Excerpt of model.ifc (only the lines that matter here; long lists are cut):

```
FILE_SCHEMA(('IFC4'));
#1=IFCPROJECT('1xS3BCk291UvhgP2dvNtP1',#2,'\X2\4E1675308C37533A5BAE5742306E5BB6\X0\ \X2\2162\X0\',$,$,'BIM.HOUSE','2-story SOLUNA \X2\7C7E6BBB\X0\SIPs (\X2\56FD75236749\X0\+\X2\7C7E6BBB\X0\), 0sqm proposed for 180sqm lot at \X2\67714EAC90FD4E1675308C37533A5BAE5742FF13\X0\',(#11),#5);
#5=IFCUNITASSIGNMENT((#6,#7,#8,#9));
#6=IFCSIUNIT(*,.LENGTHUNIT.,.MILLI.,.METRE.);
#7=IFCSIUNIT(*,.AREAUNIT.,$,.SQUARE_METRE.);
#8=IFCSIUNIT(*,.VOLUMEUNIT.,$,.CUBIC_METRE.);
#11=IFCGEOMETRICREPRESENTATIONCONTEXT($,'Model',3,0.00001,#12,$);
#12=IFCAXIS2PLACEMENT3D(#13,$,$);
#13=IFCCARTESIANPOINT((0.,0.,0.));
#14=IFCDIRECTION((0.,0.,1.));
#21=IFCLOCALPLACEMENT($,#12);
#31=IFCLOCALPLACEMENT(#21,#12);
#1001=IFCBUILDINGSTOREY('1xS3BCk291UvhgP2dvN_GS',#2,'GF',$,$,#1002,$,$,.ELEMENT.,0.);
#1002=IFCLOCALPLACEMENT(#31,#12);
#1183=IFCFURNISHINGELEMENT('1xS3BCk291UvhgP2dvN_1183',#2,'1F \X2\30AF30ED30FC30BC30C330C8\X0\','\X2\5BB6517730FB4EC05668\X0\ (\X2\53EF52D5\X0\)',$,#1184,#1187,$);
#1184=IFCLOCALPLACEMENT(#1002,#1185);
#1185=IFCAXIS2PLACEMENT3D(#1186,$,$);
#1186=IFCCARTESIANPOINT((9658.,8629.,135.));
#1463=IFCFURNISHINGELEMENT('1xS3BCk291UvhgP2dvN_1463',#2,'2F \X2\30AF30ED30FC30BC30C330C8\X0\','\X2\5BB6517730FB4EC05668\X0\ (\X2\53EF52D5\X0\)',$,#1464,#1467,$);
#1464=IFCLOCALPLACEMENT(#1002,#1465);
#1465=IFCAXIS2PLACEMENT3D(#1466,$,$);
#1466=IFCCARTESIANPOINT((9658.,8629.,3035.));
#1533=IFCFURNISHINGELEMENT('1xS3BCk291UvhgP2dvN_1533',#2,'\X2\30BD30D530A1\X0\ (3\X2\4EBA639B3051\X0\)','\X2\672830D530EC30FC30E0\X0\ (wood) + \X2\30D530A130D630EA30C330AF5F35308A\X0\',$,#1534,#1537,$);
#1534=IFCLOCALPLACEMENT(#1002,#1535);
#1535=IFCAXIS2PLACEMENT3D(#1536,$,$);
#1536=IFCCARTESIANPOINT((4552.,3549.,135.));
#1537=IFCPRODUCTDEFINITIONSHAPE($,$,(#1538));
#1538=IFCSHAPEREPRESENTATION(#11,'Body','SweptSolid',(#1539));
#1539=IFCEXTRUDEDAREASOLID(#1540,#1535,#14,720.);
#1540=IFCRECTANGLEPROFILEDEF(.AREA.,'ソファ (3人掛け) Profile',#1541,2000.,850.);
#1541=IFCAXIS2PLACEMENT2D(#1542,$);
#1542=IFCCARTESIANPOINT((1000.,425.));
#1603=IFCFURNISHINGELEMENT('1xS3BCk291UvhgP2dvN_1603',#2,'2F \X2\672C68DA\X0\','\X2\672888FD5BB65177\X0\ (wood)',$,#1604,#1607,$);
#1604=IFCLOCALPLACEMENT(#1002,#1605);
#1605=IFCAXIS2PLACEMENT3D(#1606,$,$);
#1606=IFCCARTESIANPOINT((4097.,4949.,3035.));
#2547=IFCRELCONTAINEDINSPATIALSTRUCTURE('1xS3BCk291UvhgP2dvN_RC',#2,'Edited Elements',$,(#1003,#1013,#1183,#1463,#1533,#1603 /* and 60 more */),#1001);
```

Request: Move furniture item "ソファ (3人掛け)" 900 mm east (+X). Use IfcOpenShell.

```python
import ifcopenshell
import ifcopenshell.api.geometry
import ifcopenshell.util.placement

model = ifcopenshell.open("model.ifc")

item = model.by_id(1533)
matrix = ifcopenshell.util.placement.get_local_placement(item.ObjectPlacement)
matrix[0, 3] += 900.0
ifcopenshell.api.geometry.edit_object_placement(model, product=item, matrix=matrix, is_si=False)

print(ifcopenshell.util.placement.get_local_placement(item.ObjectPlacement).round(3) + 0.0)

model.write("model-out.ifc")
```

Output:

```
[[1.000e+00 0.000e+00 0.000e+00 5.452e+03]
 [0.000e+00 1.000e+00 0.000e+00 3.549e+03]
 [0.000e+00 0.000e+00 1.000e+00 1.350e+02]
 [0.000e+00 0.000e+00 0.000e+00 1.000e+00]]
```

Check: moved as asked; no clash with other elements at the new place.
